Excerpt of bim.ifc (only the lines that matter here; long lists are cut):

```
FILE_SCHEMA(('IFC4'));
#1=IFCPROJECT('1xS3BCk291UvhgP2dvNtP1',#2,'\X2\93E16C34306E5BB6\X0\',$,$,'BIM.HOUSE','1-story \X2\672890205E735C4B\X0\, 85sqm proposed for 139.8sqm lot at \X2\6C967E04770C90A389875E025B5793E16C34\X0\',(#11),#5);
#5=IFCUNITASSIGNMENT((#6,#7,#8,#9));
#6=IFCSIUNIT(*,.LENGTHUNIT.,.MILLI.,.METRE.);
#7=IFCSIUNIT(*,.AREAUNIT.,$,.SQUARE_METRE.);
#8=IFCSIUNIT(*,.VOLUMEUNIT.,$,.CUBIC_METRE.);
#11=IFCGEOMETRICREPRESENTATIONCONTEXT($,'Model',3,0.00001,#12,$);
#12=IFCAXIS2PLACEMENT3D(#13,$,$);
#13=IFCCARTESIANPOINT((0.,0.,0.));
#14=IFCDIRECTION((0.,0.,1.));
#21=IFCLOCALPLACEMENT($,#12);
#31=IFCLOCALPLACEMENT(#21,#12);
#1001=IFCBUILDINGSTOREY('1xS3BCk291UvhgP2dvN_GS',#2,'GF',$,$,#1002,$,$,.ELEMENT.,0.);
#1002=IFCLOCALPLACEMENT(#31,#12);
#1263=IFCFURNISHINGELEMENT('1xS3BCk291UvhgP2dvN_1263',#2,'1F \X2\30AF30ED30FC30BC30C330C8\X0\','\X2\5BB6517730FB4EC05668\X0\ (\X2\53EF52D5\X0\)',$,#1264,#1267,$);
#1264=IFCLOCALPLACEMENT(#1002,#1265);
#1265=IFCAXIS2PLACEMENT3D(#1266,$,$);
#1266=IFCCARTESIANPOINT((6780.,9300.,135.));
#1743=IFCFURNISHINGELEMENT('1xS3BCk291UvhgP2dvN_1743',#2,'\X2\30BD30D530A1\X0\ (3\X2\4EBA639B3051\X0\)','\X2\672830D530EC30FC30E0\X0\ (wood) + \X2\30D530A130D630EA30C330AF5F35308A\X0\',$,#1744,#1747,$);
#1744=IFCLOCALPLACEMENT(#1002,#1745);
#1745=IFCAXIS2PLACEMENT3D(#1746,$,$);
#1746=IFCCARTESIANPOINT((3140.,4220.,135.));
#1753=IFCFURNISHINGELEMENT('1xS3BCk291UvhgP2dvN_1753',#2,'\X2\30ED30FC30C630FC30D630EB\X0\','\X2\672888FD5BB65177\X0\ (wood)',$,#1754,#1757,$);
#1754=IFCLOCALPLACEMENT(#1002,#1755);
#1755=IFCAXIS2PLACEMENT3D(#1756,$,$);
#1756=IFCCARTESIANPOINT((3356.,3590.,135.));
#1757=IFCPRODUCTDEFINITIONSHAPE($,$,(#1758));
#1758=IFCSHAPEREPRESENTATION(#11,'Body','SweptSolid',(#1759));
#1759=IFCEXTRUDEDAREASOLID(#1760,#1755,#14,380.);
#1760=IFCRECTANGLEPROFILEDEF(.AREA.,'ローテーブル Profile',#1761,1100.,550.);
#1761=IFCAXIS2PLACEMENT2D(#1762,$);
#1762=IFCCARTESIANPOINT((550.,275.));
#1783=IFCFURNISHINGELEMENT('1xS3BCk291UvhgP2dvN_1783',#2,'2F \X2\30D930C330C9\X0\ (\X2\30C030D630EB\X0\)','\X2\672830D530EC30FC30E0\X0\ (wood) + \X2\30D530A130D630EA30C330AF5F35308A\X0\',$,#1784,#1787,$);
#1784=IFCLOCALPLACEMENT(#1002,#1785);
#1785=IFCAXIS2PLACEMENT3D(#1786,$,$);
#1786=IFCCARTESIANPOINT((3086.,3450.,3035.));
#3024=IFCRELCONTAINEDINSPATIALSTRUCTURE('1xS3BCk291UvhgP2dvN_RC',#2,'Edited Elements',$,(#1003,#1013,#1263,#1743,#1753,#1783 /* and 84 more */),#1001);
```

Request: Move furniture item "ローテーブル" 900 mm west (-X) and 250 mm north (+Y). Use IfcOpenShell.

```python
import ifcopenshell
import ifcopenshell.api.geometry
import ifcopenshell.util.placement
import ifcopenshell.util.unit

model = ifcopenshell.open("bim.ifc")
unit_scale = ifcopenshell.util.unit.calculate_unit_scale(model)

item = model.by_guid("1xS3BCk291UvhgP2dvN_1753")
matrix = ifcopenshell.util.placement.get_local_placement(item.ObjectPlacement)
matrix[0, 3] -= 0.9 / unit_scale
matrix[1, 3] += 0.25 / unit_scale
ifcopenshell.api.geometry.edit_object_placement(model, product=item, matrix=matrix, is_si=False)

print(ifcopenshell.util.placement.get_local_placement(item.ObjectPlacement).round(3) + 0.0)

model.write("bim_v2.ifc")
```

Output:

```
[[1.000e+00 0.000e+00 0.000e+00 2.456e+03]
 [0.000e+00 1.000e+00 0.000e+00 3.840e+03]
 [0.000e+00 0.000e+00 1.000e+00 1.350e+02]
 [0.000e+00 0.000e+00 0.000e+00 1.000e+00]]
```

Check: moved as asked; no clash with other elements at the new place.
